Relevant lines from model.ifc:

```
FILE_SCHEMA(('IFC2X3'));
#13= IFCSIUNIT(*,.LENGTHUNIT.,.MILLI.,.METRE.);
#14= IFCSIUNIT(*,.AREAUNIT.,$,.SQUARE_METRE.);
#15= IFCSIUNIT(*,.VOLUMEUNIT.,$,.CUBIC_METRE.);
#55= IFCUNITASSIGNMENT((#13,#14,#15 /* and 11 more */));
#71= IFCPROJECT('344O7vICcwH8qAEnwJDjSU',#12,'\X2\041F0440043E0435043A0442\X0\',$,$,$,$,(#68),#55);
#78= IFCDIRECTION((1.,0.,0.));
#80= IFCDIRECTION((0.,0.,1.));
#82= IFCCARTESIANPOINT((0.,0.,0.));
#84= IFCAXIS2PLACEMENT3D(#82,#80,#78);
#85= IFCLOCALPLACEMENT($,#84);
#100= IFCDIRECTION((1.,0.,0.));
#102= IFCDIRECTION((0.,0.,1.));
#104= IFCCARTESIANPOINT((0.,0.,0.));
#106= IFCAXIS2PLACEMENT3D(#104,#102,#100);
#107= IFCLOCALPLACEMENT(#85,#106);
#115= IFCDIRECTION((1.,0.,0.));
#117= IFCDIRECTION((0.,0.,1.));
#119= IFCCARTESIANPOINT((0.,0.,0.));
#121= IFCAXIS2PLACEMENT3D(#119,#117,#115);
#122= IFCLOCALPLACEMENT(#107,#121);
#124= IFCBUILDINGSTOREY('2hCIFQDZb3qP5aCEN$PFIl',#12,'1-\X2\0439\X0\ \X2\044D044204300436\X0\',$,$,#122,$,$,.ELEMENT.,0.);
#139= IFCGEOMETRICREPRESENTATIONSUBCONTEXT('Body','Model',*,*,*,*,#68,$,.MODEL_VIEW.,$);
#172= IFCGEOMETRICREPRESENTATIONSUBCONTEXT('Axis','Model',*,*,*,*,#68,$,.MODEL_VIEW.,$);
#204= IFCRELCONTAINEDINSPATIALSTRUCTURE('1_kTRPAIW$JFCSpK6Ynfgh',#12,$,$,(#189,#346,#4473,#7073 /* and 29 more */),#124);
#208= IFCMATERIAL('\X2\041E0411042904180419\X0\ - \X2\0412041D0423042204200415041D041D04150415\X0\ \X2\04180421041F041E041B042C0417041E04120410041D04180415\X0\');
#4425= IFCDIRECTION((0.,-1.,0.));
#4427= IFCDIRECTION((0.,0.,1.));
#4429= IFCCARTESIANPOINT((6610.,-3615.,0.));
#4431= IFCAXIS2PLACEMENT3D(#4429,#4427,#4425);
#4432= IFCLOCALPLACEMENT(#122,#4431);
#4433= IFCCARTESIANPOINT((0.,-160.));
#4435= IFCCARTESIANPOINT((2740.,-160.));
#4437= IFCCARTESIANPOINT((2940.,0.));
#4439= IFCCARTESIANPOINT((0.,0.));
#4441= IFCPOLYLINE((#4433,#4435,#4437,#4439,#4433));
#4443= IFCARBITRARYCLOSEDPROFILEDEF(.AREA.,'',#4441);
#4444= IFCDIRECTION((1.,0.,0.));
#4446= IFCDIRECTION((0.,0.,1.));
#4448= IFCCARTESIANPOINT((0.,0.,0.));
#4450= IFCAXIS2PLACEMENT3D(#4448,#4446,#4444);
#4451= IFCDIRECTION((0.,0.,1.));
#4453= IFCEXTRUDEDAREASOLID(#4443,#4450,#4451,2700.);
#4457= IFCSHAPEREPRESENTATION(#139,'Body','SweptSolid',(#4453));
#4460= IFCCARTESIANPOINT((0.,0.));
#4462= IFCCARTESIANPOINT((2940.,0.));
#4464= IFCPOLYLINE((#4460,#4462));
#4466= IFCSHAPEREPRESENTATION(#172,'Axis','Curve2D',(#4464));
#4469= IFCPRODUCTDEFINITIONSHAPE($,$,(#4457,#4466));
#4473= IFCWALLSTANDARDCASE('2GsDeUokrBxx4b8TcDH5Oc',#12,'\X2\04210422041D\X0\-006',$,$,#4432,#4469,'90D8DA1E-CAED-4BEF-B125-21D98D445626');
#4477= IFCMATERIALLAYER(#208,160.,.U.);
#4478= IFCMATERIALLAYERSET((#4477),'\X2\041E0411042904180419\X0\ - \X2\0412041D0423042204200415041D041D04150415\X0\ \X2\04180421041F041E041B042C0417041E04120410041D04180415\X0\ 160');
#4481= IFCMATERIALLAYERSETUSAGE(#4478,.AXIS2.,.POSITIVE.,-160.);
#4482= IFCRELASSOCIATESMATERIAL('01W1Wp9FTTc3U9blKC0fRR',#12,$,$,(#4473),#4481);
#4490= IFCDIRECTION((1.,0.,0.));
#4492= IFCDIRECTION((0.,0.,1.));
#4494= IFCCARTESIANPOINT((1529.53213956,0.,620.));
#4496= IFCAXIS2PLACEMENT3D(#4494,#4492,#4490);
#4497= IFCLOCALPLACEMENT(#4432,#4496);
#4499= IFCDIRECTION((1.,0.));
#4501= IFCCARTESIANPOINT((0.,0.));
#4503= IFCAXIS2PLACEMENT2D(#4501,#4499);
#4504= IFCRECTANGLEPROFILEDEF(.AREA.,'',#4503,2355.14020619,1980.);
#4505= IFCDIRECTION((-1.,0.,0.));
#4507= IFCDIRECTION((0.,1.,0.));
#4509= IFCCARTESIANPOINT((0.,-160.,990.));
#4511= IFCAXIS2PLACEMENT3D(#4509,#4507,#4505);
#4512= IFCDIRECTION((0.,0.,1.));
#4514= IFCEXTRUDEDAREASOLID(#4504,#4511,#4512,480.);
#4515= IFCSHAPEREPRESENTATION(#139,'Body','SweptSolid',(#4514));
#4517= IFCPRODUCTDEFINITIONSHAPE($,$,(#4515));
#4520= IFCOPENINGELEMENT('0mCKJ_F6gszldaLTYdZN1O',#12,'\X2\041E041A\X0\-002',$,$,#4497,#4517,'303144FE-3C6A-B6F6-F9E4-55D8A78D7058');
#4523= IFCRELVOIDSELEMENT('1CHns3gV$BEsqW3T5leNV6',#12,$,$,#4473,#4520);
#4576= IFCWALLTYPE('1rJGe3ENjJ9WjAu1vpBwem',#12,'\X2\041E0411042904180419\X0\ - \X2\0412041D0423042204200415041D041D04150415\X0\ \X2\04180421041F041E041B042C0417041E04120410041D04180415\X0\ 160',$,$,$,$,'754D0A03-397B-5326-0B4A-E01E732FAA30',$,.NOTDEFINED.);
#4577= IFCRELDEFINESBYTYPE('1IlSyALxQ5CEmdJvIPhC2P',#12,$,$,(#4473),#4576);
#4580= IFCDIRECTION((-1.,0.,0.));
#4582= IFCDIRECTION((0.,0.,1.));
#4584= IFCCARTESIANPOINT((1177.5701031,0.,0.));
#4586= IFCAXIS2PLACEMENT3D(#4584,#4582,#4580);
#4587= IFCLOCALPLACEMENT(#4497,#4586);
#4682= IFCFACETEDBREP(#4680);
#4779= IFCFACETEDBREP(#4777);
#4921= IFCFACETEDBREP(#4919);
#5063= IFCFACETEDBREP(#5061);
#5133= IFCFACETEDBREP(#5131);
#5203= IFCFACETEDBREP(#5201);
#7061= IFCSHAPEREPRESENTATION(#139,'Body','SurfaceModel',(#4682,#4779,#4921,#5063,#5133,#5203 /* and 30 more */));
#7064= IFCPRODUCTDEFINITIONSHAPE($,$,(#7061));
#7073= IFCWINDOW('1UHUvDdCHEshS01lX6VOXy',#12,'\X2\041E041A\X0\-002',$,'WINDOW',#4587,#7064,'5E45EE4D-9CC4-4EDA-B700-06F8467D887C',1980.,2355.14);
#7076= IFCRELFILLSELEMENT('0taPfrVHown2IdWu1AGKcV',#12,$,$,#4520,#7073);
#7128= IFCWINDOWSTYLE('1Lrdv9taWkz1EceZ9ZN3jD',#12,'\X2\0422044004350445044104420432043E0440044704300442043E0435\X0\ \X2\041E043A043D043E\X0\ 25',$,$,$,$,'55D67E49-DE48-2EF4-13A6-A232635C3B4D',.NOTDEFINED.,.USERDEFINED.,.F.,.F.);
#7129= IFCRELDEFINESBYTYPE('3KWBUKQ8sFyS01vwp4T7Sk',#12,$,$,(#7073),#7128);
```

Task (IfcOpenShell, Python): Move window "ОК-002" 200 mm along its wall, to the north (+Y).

```python
import ifcopenshell
import ifcopenshell.api.geometry
import ifcopenshell.util.placement
import ifcopenshell.util.unit

model = ifcopenshell.open("model.ifc")
unit_scale = ifcopenshell.util.unit.calculate_unit_scale(model)

window = model.by_id(7073)
opening = window.FillsVoids[0].RelatingOpeningElement
wall = opening.VoidsElements[0].RelatingBuildingElement

wall_matrix = ifcopenshell.util.placement.get_local_placement(wall.ObjectPlacement)
shift = wall_matrix[:3, 0] * -0.2 / unit_scale
before = ifcopenshell.util.placement.get_local_placement(window.ObjectPlacement)[:3, 3].copy()

# The window is placed relative to its opening, so it follows when the opening moves.
matrix = ifcopenshell.util.placement.get_local_placement(opening.ObjectPlacement)
matrix[:3, 3] += shift
ifcopenshell.api.geometry.edit_object_placement(
    model, product=opening, matrix=matrix, is_si=False, should_transform_children=True
)

after = ifcopenshell.util.placement.get_local_placement(window.ObjectPlacement)[:3, 3]
print("window moved by", (after - before).round(3) + 0.0)

model.write("model_edited.ifc")
```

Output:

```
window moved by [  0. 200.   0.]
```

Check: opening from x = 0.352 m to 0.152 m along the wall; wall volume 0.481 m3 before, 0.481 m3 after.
